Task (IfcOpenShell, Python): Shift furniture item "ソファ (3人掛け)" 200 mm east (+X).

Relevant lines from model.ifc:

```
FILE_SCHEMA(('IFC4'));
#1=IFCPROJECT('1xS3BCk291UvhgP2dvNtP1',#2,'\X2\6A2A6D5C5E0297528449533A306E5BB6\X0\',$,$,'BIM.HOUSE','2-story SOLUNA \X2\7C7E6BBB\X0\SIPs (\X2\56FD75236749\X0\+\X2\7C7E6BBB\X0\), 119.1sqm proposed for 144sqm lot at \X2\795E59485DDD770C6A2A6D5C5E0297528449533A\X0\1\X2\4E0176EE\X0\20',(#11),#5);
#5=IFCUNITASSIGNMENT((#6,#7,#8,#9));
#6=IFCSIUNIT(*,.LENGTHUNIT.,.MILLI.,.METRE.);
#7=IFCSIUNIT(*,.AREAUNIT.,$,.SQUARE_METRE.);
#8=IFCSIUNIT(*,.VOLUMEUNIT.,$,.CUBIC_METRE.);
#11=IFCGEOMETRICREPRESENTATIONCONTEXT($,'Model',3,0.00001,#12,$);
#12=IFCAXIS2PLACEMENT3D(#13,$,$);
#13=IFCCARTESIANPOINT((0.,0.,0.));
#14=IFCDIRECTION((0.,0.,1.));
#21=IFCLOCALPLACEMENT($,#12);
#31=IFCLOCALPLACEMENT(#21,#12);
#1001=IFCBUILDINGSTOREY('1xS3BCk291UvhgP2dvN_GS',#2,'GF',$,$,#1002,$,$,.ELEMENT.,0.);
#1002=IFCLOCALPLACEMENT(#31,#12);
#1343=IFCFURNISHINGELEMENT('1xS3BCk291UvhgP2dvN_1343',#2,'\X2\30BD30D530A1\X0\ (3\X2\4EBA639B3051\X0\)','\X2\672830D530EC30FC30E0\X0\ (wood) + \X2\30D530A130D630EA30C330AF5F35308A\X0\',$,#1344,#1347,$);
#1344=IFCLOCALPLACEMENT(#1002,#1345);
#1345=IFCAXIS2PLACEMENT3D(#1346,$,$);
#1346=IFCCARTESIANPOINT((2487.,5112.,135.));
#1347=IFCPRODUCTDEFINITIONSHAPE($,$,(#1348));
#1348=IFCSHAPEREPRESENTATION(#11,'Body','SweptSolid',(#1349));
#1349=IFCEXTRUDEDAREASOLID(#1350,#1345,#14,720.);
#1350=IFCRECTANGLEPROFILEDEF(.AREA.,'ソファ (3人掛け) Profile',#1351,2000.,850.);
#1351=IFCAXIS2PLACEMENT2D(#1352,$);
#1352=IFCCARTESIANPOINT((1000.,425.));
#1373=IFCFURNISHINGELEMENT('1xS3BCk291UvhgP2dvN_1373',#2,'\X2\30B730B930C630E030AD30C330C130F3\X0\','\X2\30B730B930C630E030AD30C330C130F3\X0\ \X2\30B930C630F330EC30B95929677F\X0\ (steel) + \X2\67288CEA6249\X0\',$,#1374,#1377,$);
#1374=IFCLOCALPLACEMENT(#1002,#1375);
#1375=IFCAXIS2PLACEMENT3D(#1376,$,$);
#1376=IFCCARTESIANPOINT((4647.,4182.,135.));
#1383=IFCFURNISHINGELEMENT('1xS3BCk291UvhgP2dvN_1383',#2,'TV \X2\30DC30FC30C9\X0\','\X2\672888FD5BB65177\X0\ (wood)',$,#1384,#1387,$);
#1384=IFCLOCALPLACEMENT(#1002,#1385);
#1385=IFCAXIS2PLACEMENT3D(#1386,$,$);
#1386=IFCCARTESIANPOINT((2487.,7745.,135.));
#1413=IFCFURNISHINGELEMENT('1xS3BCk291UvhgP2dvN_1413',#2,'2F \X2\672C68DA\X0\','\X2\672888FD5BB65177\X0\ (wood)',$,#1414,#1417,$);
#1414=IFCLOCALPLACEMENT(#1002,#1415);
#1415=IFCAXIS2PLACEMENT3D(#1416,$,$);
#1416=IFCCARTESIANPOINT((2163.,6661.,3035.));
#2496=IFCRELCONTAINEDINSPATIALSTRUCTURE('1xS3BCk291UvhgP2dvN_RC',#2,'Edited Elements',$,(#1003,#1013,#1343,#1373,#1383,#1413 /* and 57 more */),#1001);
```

```python
import ifcopenshell
import ifcopenshell.api.geometry
import ifcopenshell.util.placement
import ifcopenshell.util.unit

model = ifcopenshell.open("model.ifc")
unit_scale = ifcopenshell.util.unit.calculate_unit_scale(model)

item = model.by_id(1343)
matrix = ifcopenshell.util.placement.get_local_placement(item.ObjectPlacement)
matrix[0, 3] += 0.2 / unit_scale
ifcopenshell.api.geometry.edit_object_placement(model, product=item, matrix=matrix, is_si=False)

print(ifcopenshell.util.placement.get_local_placement(item.ObjectPlacement).round(3) + 0.0)

model.write("model_updated.ifc")
```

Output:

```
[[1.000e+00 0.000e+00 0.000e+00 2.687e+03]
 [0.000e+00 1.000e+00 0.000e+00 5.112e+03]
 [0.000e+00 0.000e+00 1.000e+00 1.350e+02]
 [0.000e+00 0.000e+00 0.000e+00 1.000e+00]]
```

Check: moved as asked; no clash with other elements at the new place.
